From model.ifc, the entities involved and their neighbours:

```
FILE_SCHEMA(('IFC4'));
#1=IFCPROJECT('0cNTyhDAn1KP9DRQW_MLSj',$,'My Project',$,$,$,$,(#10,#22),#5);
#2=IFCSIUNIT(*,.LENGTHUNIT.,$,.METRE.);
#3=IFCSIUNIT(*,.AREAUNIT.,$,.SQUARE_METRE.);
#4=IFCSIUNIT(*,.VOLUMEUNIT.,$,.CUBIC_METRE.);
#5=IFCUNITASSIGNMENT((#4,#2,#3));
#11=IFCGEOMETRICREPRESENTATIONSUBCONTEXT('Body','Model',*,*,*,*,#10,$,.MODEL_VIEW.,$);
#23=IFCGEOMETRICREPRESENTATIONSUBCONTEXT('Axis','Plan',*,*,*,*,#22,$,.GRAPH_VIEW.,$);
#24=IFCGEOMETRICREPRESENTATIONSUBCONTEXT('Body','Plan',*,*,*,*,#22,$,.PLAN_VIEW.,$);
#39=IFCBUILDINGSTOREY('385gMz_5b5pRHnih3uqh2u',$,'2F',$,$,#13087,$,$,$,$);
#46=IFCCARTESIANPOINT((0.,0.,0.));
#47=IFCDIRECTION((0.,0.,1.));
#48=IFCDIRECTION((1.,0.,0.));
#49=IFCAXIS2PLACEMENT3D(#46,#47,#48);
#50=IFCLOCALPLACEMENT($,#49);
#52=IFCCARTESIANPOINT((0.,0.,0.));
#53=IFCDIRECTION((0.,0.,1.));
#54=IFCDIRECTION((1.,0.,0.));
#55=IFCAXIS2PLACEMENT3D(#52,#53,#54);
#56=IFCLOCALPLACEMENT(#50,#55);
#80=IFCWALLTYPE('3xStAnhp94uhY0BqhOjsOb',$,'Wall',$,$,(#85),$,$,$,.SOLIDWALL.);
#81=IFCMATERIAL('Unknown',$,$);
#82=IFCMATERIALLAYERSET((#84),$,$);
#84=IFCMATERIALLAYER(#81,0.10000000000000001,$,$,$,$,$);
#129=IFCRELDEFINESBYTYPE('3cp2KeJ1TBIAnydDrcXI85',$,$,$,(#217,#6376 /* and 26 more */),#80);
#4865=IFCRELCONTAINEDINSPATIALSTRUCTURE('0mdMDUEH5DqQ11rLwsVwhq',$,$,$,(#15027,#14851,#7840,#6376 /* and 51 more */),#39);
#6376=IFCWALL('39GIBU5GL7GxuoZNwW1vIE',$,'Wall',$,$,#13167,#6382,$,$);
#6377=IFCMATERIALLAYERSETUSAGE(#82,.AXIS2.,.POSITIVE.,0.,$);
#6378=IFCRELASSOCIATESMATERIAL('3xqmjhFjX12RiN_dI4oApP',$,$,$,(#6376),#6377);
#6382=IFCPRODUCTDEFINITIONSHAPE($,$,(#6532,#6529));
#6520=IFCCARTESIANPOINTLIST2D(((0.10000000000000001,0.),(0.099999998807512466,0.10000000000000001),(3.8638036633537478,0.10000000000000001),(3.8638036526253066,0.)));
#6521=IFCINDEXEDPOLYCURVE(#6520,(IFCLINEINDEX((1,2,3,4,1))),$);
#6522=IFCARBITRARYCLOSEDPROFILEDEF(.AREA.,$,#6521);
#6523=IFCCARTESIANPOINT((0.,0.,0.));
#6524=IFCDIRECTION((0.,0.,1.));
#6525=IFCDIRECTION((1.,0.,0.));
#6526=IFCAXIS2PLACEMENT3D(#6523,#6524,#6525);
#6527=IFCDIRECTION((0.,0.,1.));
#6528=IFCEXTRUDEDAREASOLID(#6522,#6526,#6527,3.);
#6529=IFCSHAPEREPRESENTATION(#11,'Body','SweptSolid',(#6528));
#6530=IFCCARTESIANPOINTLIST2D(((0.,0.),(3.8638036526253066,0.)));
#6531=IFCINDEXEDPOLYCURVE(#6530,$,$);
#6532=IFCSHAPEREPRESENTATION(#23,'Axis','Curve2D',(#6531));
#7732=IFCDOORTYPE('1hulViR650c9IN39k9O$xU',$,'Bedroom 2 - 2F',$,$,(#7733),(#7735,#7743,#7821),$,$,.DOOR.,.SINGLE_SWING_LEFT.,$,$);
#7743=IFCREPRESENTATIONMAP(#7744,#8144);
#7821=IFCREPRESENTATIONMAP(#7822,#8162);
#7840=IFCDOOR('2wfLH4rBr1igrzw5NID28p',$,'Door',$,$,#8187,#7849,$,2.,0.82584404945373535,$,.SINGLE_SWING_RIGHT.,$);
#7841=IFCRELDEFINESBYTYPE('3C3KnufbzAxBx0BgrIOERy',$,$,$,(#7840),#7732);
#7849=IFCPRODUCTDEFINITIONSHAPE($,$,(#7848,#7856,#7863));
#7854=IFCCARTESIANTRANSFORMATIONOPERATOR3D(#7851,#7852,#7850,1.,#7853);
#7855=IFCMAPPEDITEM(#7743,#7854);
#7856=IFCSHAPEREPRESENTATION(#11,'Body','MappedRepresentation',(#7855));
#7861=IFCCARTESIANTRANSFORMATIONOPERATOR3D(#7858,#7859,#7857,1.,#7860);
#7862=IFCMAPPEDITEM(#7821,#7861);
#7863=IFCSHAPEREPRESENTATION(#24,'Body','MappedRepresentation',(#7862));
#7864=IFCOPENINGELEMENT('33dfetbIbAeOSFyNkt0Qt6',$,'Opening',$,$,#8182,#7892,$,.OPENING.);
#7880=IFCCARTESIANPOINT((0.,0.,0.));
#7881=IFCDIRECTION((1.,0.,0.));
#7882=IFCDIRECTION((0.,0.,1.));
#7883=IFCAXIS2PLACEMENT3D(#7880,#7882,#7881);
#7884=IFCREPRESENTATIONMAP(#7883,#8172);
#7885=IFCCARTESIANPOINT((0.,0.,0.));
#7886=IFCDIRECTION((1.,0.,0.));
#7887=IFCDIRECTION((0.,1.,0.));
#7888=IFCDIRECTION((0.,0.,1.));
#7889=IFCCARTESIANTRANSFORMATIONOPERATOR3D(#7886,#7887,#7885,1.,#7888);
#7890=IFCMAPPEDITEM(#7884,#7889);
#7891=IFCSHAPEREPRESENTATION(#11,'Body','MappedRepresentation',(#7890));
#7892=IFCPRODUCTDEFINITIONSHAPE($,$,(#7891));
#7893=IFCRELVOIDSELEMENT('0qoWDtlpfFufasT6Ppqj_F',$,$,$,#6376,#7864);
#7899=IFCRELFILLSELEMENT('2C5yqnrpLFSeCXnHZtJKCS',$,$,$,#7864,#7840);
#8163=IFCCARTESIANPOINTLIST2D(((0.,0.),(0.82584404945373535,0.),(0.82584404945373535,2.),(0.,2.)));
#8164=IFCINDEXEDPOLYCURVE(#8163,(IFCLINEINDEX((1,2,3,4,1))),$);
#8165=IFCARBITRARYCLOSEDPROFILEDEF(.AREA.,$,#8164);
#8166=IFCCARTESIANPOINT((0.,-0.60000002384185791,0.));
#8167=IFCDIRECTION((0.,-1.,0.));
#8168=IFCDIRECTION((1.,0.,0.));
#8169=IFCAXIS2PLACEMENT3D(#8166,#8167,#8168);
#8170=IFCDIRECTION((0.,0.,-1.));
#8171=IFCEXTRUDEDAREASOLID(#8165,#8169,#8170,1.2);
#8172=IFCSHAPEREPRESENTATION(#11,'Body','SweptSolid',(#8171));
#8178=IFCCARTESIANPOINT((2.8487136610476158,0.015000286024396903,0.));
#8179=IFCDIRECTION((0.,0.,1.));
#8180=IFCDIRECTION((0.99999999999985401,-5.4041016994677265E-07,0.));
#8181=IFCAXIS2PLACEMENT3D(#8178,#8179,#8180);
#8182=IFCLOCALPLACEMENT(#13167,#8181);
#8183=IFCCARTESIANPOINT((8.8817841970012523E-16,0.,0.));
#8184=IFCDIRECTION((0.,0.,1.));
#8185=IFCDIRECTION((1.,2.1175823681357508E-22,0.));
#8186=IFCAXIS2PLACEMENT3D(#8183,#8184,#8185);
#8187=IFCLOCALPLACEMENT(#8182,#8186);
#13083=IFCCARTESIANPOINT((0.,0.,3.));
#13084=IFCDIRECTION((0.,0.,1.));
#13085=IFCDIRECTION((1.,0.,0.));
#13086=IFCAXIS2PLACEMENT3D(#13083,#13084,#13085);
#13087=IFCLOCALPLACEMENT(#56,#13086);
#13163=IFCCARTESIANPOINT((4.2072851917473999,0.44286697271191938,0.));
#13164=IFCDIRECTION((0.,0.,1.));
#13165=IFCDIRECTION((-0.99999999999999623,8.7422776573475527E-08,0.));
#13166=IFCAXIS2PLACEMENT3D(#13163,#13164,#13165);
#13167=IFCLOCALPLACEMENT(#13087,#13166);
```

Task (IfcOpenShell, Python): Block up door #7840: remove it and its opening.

```python
import ifcopenshell
import ifcopenshell.api.feature
import ifcopenshell.api.root
import ifcopenshell.geom
import ifcopenshell.util.shape

model = ifcopenshell.open("model.ifc")
settings = ifcopenshell.geom.settings()


def volume(element):
    """Net volume in cubic metres, openings subtracted."""
    shape = ifcopenshell.geom.create_shape(settings, element)
    return ifcopenshell.util.shape.get_volume(shape.geometry)


door = model.by_guid("2wfLH4rBr1igrzw5NID28p")
opening = door.FillsVoids[0].RelatingOpeningElement
wall = opening.VoidsElements[0].RelatingBuildingElement
before = volume(wall)

ifcopenshell.api.root.remove_product(model, product=door)
ifcopenshell.api.feature.remove_feature(model, feature=opening)

after = volume(wall)

print(f"wall volume {before:.3f} -> {after:.3f} m3")

model.write("model-out.ifc")
```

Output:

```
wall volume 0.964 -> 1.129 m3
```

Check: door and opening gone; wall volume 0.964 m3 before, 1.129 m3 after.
